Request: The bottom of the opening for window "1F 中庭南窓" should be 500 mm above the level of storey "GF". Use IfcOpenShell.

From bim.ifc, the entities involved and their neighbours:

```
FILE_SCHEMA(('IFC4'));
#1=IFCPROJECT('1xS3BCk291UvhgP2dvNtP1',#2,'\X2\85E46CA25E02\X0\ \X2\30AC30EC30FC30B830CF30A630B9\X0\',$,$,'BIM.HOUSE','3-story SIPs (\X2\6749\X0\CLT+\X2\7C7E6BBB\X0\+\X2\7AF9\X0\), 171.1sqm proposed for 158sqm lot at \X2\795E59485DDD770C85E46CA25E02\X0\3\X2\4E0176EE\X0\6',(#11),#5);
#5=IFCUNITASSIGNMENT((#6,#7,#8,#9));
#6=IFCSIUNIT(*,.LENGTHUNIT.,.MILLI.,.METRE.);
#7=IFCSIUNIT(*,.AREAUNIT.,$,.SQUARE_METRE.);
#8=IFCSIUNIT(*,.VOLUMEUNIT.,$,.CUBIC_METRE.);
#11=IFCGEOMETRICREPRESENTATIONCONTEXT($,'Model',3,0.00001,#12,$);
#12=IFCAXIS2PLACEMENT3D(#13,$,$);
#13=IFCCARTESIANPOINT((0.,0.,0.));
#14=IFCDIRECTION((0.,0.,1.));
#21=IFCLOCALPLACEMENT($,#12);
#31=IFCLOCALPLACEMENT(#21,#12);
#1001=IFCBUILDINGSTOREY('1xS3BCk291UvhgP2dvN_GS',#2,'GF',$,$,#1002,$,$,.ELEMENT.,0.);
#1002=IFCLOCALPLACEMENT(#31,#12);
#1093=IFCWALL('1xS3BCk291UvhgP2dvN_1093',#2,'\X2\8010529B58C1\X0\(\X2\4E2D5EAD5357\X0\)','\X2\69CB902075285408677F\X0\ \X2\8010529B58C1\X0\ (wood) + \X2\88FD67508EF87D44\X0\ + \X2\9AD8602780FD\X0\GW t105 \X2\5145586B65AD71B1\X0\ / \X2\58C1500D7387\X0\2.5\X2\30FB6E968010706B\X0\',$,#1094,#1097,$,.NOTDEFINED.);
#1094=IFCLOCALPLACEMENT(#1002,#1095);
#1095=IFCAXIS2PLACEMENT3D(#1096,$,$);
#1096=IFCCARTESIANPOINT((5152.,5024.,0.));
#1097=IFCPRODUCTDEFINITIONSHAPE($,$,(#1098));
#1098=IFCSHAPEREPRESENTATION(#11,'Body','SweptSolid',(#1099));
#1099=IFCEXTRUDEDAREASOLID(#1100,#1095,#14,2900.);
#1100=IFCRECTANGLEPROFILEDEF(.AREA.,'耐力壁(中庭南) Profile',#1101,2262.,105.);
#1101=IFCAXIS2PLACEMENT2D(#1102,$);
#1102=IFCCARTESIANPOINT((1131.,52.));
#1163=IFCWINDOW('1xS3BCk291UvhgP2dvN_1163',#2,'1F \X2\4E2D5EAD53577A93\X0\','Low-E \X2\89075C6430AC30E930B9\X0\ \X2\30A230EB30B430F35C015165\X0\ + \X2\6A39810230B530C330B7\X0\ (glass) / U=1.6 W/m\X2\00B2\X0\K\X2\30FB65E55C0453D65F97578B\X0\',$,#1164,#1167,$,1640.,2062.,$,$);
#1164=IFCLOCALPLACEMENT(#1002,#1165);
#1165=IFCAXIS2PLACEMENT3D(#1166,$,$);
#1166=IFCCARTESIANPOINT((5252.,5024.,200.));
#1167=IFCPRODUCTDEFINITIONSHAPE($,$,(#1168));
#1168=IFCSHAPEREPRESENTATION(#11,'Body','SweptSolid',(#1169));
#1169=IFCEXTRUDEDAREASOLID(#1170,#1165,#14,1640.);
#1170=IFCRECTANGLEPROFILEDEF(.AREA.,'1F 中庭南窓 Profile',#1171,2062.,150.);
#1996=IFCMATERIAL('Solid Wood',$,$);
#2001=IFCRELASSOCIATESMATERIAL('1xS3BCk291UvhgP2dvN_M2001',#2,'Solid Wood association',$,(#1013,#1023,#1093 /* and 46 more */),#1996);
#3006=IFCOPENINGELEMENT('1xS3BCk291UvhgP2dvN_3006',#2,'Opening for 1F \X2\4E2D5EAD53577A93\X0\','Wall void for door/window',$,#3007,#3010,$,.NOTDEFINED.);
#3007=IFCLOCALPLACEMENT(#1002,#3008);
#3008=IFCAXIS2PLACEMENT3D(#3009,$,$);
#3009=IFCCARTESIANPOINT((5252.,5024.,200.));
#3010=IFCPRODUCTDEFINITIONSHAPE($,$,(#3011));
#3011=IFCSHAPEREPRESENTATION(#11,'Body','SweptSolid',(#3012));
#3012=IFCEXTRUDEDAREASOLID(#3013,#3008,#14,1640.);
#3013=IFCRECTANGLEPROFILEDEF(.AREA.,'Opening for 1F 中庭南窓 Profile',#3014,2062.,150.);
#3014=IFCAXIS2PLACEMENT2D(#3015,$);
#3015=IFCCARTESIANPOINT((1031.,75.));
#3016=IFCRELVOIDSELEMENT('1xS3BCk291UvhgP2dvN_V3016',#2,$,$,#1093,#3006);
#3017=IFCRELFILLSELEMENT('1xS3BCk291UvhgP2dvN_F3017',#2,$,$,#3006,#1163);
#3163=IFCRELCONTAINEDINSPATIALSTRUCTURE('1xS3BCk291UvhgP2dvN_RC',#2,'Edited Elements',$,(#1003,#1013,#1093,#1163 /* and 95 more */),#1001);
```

```python
import numpy as np
import ifcopenshell
import ifcopenshell.api.geometry
import ifcopenshell.geom
import ifcopenshell.util.element
import ifcopenshell.util.placement
import ifcopenshell.util.shape
import ifcopenshell.util.unit

model = ifcopenshell.open("bim.ifc")
unit_scale = ifcopenshell.util.unit.calculate_unit_scale(model)

window = model.by_guid("1xS3BCk291UvhgP2dvN_1163")
opening = window.FillsVoids[0].RelatingOpeningElement
storey = ifcopenshell.util.element.get_container(window, ifc_class="IfcBuildingStorey")
level = ifcopenshell.util.placement.get_local_placement(storey.ObjectPlacement)[2, 3]

# The opening's origin need not be at the sill, so measure its lowest point.
shape = ifcopenshell.geom.create_shape(ifcopenshell.geom.settings(), opening)
bottom = ifcopenshell.util.shape.get_shape_bottom_elevation(shape, shape.geometry) / unit_scale
dz = level + 0.5 / unit_scale - bottom

shift = np.array([0.0, 0.0, dz])
# The window is not placed relative to its opening, so move both.
for product in (opening, window):
    matrix = ifcopenshell.util.placement.get_local_placement(product.ObjectPlacement)
    matrix[:3, 3] += shift
    ifcopenshell.api.geometry.edit_object_placement(model, product=product, matrix=matrix, is_si=False)

print(f"moved by {dz * unit_scale:+.3f} m")

model.write("bim_rev.ifc")
```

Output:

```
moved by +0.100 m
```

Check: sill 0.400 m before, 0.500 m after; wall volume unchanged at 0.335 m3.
